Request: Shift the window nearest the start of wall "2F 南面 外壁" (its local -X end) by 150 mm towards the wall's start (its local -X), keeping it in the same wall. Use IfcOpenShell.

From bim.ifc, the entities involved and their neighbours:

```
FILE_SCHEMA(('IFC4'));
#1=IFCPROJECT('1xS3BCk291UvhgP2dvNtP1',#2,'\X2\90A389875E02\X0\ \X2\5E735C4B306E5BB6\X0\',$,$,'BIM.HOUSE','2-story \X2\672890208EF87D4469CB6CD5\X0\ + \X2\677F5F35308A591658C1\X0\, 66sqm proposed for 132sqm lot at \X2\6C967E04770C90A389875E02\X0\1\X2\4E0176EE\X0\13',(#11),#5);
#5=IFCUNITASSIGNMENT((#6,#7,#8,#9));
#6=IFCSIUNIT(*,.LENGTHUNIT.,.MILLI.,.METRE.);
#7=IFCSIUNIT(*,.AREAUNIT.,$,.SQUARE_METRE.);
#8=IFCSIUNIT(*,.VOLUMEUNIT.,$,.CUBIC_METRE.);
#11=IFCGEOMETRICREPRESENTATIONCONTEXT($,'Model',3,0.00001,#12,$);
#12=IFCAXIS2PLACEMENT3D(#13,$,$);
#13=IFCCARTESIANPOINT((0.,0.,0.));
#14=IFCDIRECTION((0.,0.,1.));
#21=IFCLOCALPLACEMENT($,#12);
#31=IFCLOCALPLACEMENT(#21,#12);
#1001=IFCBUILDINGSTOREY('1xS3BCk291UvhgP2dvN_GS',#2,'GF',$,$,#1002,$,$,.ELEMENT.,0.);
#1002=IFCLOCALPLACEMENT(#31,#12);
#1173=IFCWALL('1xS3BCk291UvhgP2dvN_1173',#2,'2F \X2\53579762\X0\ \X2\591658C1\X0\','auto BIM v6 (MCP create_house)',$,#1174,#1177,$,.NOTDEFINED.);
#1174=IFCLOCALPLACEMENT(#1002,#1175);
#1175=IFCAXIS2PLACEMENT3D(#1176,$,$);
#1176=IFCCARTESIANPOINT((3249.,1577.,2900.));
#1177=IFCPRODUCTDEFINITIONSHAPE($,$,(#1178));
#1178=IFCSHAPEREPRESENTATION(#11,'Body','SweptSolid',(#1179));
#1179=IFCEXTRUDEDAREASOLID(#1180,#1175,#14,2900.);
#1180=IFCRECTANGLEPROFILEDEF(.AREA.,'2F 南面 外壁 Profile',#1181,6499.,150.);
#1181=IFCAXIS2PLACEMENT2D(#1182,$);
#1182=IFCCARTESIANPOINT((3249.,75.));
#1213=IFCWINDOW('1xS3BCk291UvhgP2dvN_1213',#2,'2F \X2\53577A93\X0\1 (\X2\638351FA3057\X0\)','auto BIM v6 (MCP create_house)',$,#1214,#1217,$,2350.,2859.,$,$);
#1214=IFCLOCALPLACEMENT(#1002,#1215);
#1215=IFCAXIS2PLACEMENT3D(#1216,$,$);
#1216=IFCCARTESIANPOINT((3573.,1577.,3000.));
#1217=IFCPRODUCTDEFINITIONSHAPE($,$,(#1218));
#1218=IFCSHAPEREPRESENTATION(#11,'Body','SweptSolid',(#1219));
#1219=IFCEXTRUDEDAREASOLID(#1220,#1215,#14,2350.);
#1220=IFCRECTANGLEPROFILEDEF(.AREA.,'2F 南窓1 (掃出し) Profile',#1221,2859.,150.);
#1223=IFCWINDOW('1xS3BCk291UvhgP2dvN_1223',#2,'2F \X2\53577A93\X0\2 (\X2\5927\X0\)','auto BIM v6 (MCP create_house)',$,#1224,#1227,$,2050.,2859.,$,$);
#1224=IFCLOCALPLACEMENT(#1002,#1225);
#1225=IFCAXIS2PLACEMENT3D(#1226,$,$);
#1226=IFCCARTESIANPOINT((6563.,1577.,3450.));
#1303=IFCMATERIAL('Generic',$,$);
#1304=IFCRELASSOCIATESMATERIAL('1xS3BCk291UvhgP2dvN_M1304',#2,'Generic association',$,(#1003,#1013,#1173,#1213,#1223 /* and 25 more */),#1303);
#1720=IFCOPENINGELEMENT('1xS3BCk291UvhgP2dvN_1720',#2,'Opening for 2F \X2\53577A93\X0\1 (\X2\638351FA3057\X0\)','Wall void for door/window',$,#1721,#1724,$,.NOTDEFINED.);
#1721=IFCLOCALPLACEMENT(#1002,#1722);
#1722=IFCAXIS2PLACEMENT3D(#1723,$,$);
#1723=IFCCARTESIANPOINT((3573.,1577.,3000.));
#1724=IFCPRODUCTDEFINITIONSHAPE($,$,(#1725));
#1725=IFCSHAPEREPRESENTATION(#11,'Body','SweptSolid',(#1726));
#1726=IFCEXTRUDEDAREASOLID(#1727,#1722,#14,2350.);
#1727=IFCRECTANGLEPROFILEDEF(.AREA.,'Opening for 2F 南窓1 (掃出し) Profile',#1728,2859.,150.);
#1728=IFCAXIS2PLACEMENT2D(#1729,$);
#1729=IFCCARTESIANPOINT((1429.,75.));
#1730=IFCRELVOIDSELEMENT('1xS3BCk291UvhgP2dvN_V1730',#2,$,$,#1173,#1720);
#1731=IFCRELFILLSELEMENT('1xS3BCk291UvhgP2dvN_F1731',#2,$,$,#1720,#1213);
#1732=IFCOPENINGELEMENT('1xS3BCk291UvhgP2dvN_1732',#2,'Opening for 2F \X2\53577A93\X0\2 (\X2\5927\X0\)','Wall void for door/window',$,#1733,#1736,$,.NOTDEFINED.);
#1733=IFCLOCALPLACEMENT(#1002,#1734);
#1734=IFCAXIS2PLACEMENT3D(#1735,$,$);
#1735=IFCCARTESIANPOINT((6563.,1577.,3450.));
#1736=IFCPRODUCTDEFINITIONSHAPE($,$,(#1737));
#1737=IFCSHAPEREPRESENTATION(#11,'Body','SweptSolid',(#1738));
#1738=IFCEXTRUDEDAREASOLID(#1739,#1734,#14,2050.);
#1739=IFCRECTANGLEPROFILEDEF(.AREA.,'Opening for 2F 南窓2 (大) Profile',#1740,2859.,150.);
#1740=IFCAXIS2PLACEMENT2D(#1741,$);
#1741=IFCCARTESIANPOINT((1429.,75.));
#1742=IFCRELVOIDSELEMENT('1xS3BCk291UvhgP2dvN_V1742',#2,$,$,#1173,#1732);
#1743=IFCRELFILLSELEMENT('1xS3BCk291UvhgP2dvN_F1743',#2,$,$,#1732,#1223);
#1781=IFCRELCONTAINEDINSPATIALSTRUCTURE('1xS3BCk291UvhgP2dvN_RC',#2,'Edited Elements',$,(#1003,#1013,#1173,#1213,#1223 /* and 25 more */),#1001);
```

```python
import ifcopenshell
import ifcopenshell.api.geometry
import ifcopenshell.util.placement

model = ifcopenshell.open("bim.ifc")

window = model.by_guid("1xS3BCk291UvhgP2dvN_1213")
opening = window.FillsVoids[0].RelatingOpeningElement
wall = opening.VoidsElements[0].RelatingBuildingElement

wall_matrix = ifcopenshell.util.placement.get_local_placement(wall.ObjectPlacement)
shift = wall_matrix[:3, 0] * -150.0
before = ifcopenshell.util.placement.get_local_placement(window.ObjectPlacement)[:3, 3].copy()

# The window is not placed relative to its opening, so move both.
for product in (opening, window):
    matrix = ifcopenshell.util.placement.get_local_placement(product.ObjectPlacement)
    matrix[:3, 3] += shift
    ifcopenshell.api.geometry.edit_object_placement(model, product=product, matrix=matrix, is_si=False)

after = ifcopenshell.util.placement.get_local_placement(window.ObjectPlacement)[:3, 3]
print("window moved by", (after - before).round(3) + 0.0)

model.write("bim-out.ifc")
```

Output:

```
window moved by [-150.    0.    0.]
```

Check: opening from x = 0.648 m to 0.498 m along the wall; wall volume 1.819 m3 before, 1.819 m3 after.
